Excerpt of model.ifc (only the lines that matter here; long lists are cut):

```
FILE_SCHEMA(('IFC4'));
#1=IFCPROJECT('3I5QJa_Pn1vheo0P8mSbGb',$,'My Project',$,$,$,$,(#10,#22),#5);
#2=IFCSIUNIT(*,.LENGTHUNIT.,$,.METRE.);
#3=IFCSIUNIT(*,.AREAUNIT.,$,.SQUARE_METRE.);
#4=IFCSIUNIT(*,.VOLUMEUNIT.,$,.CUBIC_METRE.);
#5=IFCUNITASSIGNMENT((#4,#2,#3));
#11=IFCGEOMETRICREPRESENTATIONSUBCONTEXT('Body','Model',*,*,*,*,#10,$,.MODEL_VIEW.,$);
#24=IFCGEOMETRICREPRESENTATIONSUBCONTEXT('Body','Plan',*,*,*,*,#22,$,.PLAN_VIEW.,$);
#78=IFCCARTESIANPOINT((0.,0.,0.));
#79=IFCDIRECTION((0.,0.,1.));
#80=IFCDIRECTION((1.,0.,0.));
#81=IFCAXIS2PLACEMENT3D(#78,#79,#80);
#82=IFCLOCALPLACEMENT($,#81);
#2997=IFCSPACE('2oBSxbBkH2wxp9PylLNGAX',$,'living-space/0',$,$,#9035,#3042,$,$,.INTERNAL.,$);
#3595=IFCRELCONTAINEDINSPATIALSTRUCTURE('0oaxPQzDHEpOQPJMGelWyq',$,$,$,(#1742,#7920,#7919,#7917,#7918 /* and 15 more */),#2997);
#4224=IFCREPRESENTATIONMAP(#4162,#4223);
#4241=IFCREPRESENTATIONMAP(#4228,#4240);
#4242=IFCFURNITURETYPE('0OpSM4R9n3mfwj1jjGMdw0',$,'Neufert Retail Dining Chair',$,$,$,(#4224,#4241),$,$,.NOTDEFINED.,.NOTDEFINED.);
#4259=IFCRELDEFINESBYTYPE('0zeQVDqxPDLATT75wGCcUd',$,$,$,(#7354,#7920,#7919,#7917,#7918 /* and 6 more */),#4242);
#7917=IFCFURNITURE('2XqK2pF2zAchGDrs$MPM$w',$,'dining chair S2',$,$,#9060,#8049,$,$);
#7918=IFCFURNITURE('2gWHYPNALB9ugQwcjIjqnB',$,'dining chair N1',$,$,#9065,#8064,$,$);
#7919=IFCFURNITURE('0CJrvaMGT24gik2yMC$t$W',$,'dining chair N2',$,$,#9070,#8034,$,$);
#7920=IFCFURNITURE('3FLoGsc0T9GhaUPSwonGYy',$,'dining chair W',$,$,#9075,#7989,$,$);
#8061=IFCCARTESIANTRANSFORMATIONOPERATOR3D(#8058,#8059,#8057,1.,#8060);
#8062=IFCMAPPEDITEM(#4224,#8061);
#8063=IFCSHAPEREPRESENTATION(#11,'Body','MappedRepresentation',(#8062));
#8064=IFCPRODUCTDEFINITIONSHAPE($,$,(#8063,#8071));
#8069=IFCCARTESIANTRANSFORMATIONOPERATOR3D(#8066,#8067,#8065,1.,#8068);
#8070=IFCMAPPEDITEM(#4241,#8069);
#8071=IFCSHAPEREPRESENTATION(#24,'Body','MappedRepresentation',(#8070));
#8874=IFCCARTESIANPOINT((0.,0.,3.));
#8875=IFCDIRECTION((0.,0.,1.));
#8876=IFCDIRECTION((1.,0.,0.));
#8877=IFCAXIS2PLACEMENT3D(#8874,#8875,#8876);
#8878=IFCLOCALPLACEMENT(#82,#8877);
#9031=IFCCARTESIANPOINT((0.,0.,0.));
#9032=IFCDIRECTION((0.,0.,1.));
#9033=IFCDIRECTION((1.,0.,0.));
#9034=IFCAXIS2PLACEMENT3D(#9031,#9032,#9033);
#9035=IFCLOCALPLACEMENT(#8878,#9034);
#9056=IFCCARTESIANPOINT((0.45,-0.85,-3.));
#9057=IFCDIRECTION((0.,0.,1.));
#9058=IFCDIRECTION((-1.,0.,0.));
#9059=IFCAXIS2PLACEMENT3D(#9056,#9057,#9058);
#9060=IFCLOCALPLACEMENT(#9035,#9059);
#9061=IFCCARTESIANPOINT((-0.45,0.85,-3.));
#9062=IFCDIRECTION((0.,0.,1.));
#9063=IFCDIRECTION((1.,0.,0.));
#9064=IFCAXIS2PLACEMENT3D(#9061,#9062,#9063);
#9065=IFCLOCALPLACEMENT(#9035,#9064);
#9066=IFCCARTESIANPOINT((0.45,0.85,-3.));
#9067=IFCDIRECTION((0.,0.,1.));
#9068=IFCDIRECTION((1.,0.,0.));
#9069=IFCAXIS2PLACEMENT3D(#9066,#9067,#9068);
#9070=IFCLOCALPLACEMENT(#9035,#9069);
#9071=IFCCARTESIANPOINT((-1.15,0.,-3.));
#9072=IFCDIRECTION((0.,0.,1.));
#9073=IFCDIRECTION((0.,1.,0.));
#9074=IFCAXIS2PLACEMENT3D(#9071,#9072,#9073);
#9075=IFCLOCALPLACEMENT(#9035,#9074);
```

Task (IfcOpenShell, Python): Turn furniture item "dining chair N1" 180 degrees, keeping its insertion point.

```python
import ifcopenshell
import ifcopenshell.api.geometry
import ifcopenshell.util.placement

model = ifcopenshell.open("model.ifc")

item = model.by_id(7918)
matrix = ifcopenshell.util.placement.get_local_placement(item.ObjectPlacement)
matrix = matrix @ ifcopenshell.util.placement.rotation(180, "Z")
ifcopenshell.api.geometry.edit_object_placement(model, product=item, matrix=matrix, is_si=False)

print(ifcopenshell.util.placement.get_local_placement(item.ObjectPlacement).round(3) + 0.0)

model.write("model-out.ifc")
```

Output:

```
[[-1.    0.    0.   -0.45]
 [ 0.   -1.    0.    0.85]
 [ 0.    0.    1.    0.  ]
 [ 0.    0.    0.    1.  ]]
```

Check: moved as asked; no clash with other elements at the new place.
